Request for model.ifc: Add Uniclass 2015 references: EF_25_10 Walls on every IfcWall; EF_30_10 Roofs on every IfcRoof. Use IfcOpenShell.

First a look at what the model holds.

```python
import ifcopenshell

model = ifcopenshell.open("model.ifc")
print(model.schema)
print("classifications:", [c.Name for c in model.by_type("IfcClassification")])
for ifc_class in ("IfcDoor", "IfcRoof", "IfcStair", "IfcWall", "IfcWindow"):
    print(ifc_class, len(model.by_type(ifc_class)))
```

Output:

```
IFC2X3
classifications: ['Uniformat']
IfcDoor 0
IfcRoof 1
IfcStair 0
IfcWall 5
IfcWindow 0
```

```python
import ifcopenshell
import ifcopenshell.api.classification

model = ifcopenshell.open("model.ifc")

# IFC2X3 requires Source and Edition and has no link from the project to the system.
system = model.create_entity("IfcClassification", Source="NBS", Edition="2015", Name="Uniclass 2015")

codes = {
    "IfcWall": ("EF_25_10", "Walls"),
    "IfcRoof": ("EF_30_10", "Roofs"),
}
for ifc_class, (code, name) in codes.items():
    products = model.by_type(ifc_class)
    ifcopenshell.api.classification.add_reference(
        model, products=products, classification=system, identification=code, name=name
    )
    print(code, len(products))

model.write("model_v2.ifc")
```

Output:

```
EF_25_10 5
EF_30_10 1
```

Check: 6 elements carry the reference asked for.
